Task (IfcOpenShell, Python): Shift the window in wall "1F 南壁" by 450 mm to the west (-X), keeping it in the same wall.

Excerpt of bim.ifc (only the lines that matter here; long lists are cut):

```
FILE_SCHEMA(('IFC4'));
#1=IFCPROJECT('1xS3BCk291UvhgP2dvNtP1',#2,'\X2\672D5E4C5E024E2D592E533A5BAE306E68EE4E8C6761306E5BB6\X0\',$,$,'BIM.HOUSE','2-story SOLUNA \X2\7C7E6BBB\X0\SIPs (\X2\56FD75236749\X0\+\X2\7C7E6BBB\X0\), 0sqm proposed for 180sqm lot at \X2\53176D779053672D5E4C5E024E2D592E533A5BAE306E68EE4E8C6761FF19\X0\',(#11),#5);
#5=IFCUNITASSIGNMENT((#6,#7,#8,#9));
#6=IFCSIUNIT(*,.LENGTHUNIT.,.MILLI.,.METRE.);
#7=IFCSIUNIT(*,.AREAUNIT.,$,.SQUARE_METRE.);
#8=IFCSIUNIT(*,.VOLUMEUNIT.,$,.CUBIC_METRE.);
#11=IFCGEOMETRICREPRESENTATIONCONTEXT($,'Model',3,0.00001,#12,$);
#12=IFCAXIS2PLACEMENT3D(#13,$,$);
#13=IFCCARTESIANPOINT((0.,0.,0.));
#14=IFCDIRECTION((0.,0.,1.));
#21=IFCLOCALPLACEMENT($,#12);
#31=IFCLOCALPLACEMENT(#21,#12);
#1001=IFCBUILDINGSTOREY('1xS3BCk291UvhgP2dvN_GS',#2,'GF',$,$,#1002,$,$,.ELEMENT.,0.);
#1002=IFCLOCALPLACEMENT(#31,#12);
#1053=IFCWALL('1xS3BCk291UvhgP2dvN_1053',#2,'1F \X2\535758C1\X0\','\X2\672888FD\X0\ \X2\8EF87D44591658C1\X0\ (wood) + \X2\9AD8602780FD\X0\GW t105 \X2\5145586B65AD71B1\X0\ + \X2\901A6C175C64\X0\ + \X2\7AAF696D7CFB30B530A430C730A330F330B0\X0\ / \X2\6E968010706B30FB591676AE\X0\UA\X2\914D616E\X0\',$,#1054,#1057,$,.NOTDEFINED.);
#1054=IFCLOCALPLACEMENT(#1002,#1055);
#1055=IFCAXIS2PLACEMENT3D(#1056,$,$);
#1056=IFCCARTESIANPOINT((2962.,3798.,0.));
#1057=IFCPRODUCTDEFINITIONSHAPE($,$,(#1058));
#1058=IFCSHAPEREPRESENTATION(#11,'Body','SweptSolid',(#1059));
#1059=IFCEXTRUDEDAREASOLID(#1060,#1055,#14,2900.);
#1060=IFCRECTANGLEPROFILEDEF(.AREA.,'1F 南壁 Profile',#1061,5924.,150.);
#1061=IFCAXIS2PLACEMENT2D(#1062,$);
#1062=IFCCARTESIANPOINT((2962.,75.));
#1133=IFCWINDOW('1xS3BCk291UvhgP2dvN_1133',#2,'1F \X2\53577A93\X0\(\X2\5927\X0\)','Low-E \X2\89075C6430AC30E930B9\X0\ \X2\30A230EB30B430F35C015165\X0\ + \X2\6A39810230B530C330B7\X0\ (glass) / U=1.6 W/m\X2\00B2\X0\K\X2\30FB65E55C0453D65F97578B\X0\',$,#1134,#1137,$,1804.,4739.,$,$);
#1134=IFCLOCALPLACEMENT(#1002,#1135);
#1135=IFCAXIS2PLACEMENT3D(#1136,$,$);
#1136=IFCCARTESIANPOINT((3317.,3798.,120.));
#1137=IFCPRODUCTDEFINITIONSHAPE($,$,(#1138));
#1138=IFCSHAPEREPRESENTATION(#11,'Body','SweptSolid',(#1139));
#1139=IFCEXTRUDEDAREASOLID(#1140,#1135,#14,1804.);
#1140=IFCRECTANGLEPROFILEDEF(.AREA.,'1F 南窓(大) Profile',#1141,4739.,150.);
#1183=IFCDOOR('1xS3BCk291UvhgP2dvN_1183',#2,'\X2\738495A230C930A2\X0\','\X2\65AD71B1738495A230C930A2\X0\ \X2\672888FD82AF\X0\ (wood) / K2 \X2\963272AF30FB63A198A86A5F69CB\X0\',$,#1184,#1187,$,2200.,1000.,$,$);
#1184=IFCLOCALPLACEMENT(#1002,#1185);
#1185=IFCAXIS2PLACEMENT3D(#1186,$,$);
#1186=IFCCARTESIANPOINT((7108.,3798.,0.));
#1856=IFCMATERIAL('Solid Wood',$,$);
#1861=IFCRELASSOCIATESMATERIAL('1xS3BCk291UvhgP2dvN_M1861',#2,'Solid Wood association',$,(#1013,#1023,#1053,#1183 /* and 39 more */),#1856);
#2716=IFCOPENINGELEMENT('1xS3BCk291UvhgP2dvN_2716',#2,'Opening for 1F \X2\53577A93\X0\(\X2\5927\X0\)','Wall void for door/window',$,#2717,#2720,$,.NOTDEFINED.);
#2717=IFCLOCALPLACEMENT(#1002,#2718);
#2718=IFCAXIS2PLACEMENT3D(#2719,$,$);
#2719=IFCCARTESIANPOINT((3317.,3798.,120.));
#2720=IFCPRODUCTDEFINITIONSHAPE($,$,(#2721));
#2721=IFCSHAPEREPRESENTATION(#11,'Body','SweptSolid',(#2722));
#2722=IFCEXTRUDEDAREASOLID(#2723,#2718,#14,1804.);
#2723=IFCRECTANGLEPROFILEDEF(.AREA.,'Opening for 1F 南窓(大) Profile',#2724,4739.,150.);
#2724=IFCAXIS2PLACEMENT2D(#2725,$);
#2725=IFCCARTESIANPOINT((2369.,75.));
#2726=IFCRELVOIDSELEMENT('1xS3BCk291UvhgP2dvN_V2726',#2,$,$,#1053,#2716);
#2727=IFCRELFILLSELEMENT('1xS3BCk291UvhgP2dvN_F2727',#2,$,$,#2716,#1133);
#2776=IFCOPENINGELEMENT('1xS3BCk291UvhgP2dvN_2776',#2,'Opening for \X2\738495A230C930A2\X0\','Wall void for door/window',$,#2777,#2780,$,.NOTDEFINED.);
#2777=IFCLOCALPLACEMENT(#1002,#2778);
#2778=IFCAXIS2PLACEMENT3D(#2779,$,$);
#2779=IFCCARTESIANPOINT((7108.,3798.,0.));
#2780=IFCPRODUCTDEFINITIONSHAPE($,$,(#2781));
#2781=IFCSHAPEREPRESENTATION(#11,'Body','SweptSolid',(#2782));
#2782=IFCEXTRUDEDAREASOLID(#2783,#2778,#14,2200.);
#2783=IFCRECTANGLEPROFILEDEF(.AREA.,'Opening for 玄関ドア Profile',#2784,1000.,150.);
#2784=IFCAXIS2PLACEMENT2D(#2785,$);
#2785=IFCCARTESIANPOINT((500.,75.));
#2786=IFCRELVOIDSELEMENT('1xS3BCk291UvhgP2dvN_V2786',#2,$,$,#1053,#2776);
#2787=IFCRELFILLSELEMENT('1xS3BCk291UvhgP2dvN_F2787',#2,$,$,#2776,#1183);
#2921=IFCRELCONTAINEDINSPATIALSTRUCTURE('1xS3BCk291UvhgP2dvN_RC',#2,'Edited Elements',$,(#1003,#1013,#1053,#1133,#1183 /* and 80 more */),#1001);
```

```python
import ifcopenshell
import ifcopenshell.api.geometry
import ifcopenshell.util.placement
import ifcopenshell.util.unit

model = ifcopenshell.open("bim.ifc")
unit_scale = ifcopenshell.util.unit.calculate_unit_scale(model)

window = model.by_id(1133)
opening = window.FillsVoids[0].RelatingOpeningElement
wall = opening.VoidsElements[0].RelatingBuildingElement

wall_matrix = ifcopenshell.util.placement.get_local_placement(wall.ObjectPlacement)
shift = wall_matrix[:3, 0] * -0.45 / unit_scale
before = ifcopenshell.util.placement.get_local_placement(window.ObjectPlacement)[:3, 3].copy()

# The window is not placed relative to its opening, so move both.
for product in (opening, window):
    matrix = ifcopenshell.util.placement.get_local_placement(product.ObjectPlacement)
    matrix[:3, 3] += shift
    ifcopenshell.api.geometry.edit_object_placement(model, product=product, matrix=matrix, is_si=False)

after = ifcopenshell.util.placement.get_local_placement(window.ObjectPlacement)[:3, 3]
print("window moved by", (after - before).round(3) + 0.0)

model.write("bim_updated.ifc")
```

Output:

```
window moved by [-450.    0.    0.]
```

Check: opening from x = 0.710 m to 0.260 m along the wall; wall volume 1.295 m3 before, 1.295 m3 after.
